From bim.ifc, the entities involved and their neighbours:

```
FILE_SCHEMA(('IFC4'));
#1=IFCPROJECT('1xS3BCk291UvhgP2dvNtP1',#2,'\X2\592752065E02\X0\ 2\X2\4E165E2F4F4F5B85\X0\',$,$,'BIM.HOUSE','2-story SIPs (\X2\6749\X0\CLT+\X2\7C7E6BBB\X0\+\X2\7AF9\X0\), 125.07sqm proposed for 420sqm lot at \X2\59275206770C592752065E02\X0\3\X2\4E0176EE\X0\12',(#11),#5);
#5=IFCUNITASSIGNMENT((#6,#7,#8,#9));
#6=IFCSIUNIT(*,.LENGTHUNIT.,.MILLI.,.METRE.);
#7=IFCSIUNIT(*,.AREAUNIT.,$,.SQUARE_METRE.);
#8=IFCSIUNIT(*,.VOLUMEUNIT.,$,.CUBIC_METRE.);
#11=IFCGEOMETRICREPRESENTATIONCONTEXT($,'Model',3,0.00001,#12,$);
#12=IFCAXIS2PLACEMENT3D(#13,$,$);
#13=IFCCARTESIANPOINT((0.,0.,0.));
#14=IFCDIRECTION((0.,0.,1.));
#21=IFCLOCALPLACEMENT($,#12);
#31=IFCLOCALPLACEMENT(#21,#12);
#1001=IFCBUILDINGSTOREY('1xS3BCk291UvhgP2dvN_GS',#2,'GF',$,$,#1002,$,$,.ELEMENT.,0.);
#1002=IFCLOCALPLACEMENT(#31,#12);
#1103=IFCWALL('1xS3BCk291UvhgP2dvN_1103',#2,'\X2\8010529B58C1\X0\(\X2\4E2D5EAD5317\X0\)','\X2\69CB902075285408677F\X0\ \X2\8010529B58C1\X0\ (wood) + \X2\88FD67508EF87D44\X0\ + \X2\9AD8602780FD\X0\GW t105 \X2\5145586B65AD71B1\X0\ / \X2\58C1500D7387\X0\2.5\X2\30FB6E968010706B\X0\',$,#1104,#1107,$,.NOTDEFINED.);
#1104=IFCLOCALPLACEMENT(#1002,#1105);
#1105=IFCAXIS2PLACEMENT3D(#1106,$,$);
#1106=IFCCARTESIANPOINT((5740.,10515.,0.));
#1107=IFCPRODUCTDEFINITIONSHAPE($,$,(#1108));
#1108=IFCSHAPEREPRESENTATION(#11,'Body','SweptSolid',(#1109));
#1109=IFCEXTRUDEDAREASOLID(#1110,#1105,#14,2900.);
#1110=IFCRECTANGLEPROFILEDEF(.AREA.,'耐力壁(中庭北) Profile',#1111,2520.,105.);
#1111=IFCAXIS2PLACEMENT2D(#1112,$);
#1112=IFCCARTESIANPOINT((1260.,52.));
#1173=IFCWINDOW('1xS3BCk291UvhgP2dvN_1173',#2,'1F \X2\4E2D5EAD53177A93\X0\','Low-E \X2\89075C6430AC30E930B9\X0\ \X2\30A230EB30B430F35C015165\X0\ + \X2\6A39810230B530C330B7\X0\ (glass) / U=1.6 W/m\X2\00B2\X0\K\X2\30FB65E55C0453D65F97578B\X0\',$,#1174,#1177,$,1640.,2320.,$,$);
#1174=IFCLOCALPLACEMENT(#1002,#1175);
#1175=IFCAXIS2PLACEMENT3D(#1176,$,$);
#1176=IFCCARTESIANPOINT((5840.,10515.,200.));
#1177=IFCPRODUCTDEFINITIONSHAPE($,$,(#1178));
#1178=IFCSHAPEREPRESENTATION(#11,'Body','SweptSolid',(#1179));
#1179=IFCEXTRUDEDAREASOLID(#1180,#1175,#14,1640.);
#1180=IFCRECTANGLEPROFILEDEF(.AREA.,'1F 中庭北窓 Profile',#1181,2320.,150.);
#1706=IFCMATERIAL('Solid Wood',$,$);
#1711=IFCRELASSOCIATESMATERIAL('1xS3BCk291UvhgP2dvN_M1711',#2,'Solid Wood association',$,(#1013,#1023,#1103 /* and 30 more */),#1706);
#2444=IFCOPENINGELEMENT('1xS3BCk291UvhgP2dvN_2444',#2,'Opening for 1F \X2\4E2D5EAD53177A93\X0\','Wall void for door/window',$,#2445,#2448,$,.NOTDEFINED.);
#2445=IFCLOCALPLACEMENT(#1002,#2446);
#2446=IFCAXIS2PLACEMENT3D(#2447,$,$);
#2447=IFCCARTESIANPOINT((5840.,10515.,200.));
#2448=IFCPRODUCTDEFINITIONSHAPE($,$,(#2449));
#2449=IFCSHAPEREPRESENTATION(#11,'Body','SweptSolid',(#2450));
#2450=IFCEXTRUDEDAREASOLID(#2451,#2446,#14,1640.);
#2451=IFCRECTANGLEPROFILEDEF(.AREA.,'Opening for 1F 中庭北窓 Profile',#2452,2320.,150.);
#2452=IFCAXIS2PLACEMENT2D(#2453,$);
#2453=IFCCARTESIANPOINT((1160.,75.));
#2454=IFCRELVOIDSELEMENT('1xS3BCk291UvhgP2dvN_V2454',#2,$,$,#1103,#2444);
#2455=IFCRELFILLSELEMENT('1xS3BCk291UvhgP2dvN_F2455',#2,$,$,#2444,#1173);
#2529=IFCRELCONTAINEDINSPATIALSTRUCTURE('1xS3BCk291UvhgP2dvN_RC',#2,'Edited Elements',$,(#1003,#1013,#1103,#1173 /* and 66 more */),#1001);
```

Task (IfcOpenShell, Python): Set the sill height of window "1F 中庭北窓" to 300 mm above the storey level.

```python
import numpy as np
import ifcopenshell
import ifcopenshell.api.geometry
import ifcopenshell.geom
import ifcopenshell.util.element
import ifcopenshell.util.placement
import ifcopenshell.util.shape
import ifcopenshell.util.unit

model = ifcopenshell.open("bim.ifc")
unit_scale = ifcopenshell.util.unit.calculate_unit_scale(model)

window = model.by_guid("1xS3BCk291UvhgP2dvN_1173")
opening = window.FillsVoids[0].RelatingOpeningElement
storey = ifcopenshell.util.element.get_container(window, ifc_class="IfcBuildingStorey")
level = ifcopenshell.util.placement.get_local_placement(storey.ObjectPlacement)[2, 3]

# The opening's origin need not be at the sill, so measure its lowest point.
shape = ifcopenshell.geom.create_shape(ifcopenshell.geom.settings(), opening)
bottom = ifcopenshell.util.shape.get_shape_bottom_elevation(shape, shape.geometry) / unit_scale
dz = level + 300.0 - bottom

shift = np.array([0.0, 0.0, dz])
# The window is not placed relative to its opening, so move both.
for product in (opening, window):
    matrix = ifcopenshell.util.placement.get_local_placement(product.ObjectPlacement)
    matrix[:3, 3] += shift
    ifcopenshell.api.geometry.edit_object_placement(model, product=product, matrix=matrix, is_si=False)

print(f"moved by {dz * unit_scale:+.3f} m")

model.write("bim-out.ifc")
```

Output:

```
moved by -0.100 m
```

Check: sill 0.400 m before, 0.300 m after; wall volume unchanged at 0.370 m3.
